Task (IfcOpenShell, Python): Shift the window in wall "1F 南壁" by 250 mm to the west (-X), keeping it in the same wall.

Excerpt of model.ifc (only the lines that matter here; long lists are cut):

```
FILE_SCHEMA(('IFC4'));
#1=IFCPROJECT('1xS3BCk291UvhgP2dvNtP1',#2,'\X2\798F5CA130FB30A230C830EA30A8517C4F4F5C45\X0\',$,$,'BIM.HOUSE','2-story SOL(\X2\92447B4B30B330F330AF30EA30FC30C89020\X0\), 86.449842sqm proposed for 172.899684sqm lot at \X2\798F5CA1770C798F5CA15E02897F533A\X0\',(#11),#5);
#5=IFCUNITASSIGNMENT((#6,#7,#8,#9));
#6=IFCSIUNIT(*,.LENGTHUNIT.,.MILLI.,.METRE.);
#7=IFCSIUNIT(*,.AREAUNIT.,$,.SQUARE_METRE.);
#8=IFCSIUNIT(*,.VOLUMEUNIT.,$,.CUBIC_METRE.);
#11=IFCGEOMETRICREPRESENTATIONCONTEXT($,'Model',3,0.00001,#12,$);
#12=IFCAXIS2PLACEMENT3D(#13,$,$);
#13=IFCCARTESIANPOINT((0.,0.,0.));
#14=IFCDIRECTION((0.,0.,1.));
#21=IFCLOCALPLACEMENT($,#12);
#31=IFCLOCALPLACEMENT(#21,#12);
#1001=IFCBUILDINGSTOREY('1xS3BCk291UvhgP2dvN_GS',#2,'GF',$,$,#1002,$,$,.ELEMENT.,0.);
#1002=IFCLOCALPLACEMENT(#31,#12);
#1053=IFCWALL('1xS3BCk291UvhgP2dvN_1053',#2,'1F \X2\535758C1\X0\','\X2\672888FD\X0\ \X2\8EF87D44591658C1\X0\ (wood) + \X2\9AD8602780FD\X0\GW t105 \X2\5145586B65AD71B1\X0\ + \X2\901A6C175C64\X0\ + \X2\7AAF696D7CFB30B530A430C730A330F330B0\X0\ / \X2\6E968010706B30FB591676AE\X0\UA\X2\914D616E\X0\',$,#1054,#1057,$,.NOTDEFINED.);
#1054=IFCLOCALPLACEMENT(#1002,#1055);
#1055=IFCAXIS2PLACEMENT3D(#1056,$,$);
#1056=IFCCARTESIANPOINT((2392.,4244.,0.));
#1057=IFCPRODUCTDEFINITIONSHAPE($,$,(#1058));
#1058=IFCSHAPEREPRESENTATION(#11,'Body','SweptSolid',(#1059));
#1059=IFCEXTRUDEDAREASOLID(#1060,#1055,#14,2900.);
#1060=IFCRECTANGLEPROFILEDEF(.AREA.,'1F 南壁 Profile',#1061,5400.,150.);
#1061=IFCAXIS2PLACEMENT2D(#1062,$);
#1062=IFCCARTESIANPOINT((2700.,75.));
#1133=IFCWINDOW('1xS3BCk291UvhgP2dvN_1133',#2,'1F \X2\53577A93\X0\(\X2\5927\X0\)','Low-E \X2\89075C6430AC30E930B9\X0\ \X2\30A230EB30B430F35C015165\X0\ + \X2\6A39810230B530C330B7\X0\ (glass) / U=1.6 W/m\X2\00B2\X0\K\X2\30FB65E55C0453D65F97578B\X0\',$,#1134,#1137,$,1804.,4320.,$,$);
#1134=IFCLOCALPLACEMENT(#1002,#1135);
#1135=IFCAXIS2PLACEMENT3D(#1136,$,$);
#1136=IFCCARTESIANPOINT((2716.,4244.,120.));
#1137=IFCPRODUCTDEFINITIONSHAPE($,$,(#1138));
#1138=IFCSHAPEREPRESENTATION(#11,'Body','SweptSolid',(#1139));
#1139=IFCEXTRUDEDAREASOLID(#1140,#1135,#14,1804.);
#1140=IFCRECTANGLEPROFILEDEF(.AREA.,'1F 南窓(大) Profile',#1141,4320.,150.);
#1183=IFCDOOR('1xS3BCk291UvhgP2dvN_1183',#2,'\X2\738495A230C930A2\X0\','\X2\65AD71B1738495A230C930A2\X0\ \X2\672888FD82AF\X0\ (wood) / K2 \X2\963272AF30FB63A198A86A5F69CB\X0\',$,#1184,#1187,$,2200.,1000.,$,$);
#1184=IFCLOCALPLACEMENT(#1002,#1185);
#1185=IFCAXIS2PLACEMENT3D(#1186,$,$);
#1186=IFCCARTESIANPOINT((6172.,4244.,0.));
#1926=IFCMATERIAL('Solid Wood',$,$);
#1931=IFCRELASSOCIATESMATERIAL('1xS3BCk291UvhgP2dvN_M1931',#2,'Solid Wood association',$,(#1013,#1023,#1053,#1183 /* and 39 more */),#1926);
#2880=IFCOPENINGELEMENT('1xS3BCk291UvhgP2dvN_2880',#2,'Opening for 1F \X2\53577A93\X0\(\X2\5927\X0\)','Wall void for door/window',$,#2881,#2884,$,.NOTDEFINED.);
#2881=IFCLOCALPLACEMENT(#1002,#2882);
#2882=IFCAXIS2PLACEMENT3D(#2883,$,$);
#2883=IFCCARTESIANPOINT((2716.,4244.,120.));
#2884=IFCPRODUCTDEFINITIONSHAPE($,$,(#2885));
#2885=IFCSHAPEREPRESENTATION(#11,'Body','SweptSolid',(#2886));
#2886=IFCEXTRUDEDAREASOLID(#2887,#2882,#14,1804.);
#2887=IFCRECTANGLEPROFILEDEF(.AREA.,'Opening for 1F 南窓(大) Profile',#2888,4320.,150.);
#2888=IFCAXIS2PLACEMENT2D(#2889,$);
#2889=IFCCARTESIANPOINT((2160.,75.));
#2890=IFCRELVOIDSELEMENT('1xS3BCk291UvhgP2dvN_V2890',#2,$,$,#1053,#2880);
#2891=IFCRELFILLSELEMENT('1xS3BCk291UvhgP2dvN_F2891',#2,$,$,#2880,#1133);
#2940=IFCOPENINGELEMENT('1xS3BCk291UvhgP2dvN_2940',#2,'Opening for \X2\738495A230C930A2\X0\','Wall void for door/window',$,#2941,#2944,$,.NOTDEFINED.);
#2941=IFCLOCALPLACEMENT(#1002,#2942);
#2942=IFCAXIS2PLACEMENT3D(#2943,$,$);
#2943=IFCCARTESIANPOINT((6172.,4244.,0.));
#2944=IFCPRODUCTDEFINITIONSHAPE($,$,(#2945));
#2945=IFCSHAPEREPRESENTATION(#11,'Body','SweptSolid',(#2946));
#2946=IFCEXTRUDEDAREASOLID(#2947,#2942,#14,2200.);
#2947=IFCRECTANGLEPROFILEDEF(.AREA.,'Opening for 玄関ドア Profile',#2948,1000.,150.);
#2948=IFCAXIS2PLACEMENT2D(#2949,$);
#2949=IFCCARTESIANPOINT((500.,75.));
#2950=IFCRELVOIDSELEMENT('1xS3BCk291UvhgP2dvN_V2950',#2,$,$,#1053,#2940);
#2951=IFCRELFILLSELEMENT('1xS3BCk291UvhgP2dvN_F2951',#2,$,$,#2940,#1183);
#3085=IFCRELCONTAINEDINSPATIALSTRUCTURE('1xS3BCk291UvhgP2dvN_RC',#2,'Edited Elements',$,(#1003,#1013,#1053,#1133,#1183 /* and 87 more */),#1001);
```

```python
import ifcopenshell
import ifcopenshell.api.geometry
import ifcopenshell.util.placement
import ifcopenshell.util.unit

model = ifcopenshell.open("model.ifc")
unit_scale = ifcopenshell.util.unit.calculate_unit_scale(model)

window = model.by_guid("1xS3BCk291UvhgP2dvN_1133")
opening = window.FillsVoids[0].RelatingOpeningElement
wall = opening.VoidsElements[0].RelatingBuildingElement

wall_matrix = ifcopenshell.util.placement.get_local_placement(wall.ObjectPlacement)
shift = wall_matrix[:3, 0] * -0.25 / unit_scale
before = ifcopenshell.util.placement.get_local_placement(window.ObjectPlacement)[:3, 3].copy()

# The window is not placed relative to its opening, so move both.
for product in (opening, window):
    matrix = ifcopenshell.util.placement.get_local_placement(product.ObjectPlacement)
    matrix[:3, 3] += shift
    ifcopenshell.api.geometry.edit_object_placement(model, product=product, matrix=matrix, is_si=False)

after = ifcopenshell.util.placement.get_local_placement(window.ObjectPlacement)[:3, 3]
print("window moved by", (after - before).round(3) + 0.0)

model.write("model_updated.ifc")
```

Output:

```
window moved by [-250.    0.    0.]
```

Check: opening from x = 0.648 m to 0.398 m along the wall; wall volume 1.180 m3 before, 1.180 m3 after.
